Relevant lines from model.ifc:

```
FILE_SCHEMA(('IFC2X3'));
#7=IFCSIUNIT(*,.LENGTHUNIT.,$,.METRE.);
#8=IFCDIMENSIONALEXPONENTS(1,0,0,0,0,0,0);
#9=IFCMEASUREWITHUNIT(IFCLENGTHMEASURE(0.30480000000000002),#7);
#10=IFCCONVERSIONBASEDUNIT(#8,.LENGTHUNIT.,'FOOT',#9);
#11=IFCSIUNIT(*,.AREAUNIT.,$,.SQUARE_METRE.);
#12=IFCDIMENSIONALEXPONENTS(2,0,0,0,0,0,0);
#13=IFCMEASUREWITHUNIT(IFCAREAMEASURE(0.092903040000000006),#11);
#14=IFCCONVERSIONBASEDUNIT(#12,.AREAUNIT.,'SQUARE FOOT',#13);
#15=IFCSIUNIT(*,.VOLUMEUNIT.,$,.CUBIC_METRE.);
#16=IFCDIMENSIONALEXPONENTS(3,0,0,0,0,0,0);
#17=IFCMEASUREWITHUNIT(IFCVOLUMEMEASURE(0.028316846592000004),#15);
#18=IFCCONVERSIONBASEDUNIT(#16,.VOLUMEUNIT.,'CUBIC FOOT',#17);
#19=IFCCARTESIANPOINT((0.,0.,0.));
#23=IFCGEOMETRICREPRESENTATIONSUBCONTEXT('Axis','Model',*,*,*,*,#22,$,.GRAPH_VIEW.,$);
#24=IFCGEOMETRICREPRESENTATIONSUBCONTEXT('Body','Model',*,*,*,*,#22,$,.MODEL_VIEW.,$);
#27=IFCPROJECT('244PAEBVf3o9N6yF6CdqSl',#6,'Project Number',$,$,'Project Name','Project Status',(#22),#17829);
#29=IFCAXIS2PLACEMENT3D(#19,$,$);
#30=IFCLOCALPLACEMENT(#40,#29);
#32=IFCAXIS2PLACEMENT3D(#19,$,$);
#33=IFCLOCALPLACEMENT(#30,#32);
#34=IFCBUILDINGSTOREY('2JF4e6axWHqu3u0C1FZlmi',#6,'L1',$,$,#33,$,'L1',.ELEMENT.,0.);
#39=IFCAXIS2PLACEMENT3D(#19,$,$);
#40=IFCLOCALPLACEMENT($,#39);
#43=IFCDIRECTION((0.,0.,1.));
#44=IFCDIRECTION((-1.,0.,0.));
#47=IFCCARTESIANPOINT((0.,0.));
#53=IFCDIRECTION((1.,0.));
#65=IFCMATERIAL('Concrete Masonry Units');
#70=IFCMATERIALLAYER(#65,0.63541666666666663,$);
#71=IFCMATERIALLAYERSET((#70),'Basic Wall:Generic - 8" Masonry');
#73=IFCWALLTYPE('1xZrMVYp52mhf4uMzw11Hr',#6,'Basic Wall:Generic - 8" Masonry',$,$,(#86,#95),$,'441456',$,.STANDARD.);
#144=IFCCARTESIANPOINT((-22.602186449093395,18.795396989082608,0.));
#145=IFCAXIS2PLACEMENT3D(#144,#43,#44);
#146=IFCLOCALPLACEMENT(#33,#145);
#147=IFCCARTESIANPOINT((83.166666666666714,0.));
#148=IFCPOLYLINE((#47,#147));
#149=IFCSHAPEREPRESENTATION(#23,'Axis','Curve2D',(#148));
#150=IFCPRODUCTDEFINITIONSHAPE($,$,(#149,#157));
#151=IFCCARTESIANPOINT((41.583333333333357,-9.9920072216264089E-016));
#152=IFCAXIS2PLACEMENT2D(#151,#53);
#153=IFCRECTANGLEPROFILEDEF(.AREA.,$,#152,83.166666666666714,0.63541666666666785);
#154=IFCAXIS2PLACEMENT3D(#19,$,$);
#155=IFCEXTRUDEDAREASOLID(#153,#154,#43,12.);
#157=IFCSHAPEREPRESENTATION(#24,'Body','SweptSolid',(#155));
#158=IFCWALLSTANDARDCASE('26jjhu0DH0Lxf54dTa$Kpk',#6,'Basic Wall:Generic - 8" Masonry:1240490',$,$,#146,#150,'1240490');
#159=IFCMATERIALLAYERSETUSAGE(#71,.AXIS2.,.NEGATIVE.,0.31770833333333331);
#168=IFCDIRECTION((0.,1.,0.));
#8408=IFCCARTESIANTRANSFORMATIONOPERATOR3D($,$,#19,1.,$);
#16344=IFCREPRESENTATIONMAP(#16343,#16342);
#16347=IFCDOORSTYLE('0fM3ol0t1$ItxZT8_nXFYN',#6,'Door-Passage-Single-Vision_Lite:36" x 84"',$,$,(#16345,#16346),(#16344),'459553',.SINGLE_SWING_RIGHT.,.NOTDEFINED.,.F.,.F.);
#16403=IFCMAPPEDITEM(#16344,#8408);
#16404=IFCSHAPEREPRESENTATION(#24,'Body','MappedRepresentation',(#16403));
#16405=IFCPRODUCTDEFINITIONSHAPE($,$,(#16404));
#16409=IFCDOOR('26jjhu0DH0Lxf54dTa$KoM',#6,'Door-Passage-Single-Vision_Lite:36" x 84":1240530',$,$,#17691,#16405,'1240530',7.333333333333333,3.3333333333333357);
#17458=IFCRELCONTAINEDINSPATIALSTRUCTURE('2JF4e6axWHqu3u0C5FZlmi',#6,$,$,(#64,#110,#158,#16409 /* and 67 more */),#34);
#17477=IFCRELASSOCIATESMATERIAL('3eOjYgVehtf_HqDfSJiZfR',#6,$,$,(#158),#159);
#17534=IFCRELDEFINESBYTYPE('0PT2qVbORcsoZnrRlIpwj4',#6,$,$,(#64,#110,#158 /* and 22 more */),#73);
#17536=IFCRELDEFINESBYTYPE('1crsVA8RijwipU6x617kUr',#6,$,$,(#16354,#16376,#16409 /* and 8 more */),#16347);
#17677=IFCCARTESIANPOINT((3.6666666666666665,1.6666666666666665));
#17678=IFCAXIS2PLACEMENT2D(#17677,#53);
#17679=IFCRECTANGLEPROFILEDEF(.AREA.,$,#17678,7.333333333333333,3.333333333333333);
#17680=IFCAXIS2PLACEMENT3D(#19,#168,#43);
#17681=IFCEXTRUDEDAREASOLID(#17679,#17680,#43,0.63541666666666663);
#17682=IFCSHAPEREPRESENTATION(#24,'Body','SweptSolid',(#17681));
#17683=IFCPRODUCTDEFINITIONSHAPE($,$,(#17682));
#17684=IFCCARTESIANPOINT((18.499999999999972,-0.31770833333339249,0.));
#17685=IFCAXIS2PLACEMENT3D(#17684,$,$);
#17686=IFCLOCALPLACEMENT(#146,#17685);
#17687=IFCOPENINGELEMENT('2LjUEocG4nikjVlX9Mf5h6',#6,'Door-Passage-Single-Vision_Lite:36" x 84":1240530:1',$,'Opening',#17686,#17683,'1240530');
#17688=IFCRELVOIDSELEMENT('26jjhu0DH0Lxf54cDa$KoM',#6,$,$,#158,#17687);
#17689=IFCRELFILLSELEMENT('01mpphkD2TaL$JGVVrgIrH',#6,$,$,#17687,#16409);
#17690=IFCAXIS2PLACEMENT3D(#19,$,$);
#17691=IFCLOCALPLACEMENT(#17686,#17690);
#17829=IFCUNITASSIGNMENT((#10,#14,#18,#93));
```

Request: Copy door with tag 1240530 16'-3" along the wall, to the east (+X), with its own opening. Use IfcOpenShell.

```python
import ifcopenshell
import ifcopenshell.api.feature
import ifcopenshell.api.geometry
import ifcopenshell.api.root
import ifcopenshell.geom
import ifcopenshell.util.element
import ifcopenshell.util.placement
import ifcopenshell.util.shape
import ifcopenshell.util.unit

model = ifcopenshell.open("model.ifc")
unit_scale = ifcopenshell.util.unit.calculate_unit_scale(model)
settings = ifcopenshell.geom.settings()


def volume(element):
    """Net volume in cubic metres, openings subtracted."""
    shape = ifcopenshell.geom.create_shape(settings, element)
    return ifcopenshell.util.shape.get_volume(shape.geometry)


def reuse_history(source, copy):
    """copy_class also copies each property set's owner history, people and application; keep the originals."""
    for rel in copy.IsDefinedBy:
        if rel.is_a("IfcRelDefinesByProperties") and (history := rel.RelatingPropertyDefinition.OwnerHistory):
            rel.RelatingPropertyDefinition.OwnerHistory = source.OwnerHistory
            ifcopenshell.util.element.remove_deep2(model, history)


door = model.by_id(16409)
opening = door.FillsVoids[0].RelatingOpeningElement
wall = opening.VoidsElements[0].RelatingBuildingElement
before = volume(wall)
shift = ifcopenshell.util.placement.get_local_placement(wall.ObjectPlacement)[:3, 0] * -195 * 0.0254 / unit_scale

# copy_class copies the void relationship, type, container and properties, but no geometry.
new_opening = ifcopenshell.api.root.copy_class(model, product=opening)
new_opening.Representation = ifcopenshell.util.element.copy_deep(
    model, opening.Representation, exclude=["IfcGeometricRepresentationContext", "IfcRepresentationMap"]
)
new_opening.Name = 'Door-Passage-Single-Vision_Lite:36" x 84"'
new_opening.Tag = None
new_door = ifcopenshell.api.root.copy_class(model, product=door)
new_door.Representation = ifcopenshell.util.element.copy_deep(
    model, door.Representation, exclude=["IfcGeometricRepresentationContext", "IfcRepresentationMap"]
)
new_door.Name = 'Door-Passage-Single-Vision_Lite:36" x 84"'
new_door.Tag = None
reuse_history(door, new_door)
fills = ifcopenshell.api.feature.add_filling(model, opening=new_opening, element=new_door)
fills.OwnerHistory = new_door.OwnerHistory  # required in IFC2X3

for old, new in ((opening, new_opening), (door, new_door)):
    matrix = ifcopenshell.util.placement.get_local_placement(old.ObjectPlacement)
    matrix[:3, 3] += shift
    ifcopenshell.api.geometry.edit_object_placement(model, product=new, matrix=matrix, is_si=False)

after = volume(wall)

print(f"wall volume {before:.3f} -> {after:.3f} m3")

model.write("model_v2.ifc")
```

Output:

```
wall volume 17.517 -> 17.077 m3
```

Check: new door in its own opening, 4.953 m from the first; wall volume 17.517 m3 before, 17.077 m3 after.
